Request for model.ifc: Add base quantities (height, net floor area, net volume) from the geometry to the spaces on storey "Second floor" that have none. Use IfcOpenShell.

First a look at what the model holds.

```python
import ifcopenshell
import ifcopenshell.util.element
import ifcopenshell.util.unit

model = ifcopenshell.open("model.ifc")
print(model.schema)
for unit_type in ("LENGTHUNIT", "AREAUNIT", "VOLUMEUNIT"):
    print(unit_type, ifcopenshell.util.unit.calculate_unit_scale(model, unit_type))
storey = next(s for s in model.by_type("IfcBuildingStorey") if s.Name == "Second floor")
spaces = [e for e in ifcopenshell.util.element.get_decomposition(storey) if e.is_a("IfcSpace")]
for e in sorted(spaces, key=lambda e: e.id()):
    print(e.id(), e.is_a(), e.Name, list(ifcopenshell.util.element.get_psets(e, qtos_only=True)), sep=" | ")
```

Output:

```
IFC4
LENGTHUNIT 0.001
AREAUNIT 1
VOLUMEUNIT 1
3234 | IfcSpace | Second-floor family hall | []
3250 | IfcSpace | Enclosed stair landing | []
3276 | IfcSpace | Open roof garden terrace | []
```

```python
import ifcopenshell
import ifcopenshell.api.pset
import ifcopenshell.geom
import ifcopenshell.util.element
import ifcopenshell.util.shape
import ifcopenshell.util.unit

model = ifcopenshell.open("model.ifc")
unit_scale = ifcopenshell.util.unit.calculate_unit_scale(model)
area_scale = ifcopenshell.util.unit.calculate_unit_scale(model, "AREAUNIT")
volume_scale = ifcopenshell.util.unit.calculate_unit_scale(model, "VOLUMEUNIT")
settings = ifcopenshell.geom.settings()

storey = next(s for s in model.by_type("IfcBuildingStorey") if s.Name == "Second floor")
spaces = [e for e in ifcopenshell.util.element.get_decomposition(storey) if e.is_a("IfcSpace")]

for e in sorted(spaces, key=lambda e: e.id()):
    if ifcopenshell.util.element.get_psets(e, qtos_only=True, should_inherit=False):
        continue
    # Geometry comes back in metres, in the element's own axes.
    shape = ifcopenshell.geom.create_shape(settings, e)
    values = {
        "Height": ifcopenshell.util.shape.get_z(shape.geometry) / unit_scale,
        "NetFloorArea": ifcopenshell.util.shape.get_footprint_area(shape.geometry) / area_scale,
        "NetVolume": ifcopenshell.util.shape.get_volume(shape.geometry) / volume_scale,
    }
    qto = ifcopenshell.api.pset.add_qto(model, product=e, name="Qto_SpaceBaseQuantities")
    ifcopenshell.api.pset.edit_qto(model, qto=qto, properties=values)
    print(e.id(), {k: round(v, 3) for k, v in values.items()})

model.write("model_v2.ifc")
```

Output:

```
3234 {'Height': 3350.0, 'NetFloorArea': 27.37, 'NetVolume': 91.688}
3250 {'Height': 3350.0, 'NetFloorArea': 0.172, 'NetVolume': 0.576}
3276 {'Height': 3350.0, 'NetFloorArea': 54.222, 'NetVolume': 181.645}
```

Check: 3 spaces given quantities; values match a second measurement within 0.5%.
